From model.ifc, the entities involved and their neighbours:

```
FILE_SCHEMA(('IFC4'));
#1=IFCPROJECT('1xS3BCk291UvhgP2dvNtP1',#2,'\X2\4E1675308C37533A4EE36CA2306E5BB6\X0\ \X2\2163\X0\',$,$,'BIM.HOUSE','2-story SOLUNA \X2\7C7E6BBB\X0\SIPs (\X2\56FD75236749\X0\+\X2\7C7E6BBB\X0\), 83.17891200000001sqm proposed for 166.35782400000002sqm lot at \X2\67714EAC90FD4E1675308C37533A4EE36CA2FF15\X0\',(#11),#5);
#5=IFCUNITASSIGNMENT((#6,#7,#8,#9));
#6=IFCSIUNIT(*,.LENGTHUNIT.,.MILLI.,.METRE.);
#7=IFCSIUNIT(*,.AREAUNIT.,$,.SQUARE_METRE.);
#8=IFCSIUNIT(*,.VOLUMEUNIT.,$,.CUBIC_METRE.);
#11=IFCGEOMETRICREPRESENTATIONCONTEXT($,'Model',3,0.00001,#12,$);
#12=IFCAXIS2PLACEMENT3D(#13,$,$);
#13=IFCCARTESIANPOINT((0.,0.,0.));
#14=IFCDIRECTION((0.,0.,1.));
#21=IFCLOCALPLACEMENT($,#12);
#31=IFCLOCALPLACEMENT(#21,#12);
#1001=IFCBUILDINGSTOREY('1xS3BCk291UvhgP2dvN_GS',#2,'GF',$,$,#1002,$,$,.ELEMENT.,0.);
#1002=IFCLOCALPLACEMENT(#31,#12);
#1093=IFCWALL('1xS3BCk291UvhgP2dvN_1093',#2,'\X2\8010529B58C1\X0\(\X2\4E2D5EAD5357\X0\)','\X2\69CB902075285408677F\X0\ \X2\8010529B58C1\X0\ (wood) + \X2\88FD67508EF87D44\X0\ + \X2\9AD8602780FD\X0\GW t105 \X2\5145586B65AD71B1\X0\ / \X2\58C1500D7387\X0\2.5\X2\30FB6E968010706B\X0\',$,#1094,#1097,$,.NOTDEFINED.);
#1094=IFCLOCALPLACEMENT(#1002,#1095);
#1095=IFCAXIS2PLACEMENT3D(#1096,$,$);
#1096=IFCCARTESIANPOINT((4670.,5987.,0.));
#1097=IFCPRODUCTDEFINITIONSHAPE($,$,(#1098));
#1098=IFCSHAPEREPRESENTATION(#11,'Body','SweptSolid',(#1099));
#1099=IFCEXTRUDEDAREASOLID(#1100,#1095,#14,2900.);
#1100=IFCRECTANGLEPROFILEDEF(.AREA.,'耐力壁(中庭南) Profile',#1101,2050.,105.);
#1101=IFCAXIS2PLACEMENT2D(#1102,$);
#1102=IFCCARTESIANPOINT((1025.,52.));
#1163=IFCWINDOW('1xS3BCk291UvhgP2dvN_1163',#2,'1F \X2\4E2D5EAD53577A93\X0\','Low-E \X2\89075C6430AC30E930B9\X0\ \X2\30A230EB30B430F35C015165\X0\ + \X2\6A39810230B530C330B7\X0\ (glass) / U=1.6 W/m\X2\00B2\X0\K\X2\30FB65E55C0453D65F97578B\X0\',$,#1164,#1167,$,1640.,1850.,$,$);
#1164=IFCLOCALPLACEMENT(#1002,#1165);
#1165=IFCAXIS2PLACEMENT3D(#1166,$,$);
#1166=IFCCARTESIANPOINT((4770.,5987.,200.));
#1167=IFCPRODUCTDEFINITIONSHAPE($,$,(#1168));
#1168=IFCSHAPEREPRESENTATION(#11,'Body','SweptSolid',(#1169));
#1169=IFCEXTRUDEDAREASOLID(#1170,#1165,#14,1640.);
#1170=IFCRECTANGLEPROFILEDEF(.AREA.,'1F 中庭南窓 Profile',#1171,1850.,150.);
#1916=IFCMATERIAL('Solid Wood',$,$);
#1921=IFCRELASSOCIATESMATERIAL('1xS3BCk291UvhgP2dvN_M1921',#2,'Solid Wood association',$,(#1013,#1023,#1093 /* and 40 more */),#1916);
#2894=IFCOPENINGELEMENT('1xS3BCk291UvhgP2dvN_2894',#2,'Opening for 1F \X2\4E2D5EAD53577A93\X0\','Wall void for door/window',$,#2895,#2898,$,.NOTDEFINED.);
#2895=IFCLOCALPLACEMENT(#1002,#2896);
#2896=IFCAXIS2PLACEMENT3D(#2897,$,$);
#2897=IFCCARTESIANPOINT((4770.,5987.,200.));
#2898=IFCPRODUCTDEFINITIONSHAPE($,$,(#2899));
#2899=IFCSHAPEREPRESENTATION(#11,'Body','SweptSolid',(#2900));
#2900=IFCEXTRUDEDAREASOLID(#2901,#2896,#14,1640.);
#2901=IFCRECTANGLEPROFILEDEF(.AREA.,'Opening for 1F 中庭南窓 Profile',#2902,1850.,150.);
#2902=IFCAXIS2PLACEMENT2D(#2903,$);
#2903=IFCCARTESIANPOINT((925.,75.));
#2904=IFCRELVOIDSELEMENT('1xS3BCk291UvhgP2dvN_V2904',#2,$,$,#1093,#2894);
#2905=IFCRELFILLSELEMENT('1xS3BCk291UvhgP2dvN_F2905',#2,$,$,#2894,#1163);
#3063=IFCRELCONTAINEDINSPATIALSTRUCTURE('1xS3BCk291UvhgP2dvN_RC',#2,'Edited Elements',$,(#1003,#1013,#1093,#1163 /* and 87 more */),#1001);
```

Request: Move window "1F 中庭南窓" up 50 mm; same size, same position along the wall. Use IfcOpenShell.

```python
import numpy as np
import ifcopenshell
import ifcopenshell.api.geometry
import ifcopenshell.util.placement
import ifcopenshell.util.unit

model = ifcopenshell.open("model.ifc")
unit_scale = ifcopenshell.util.unit.calculate_unit_scale(model)

window = model.by_id(1163)
opening = window.FillsVoids[0].RelatingOpeningElement
dz = 0.05 / unit_scale

shift = np.array([0.0, 0.0, dz])
# The window is not placed relative to its opening, so move both.
for product in (opening, window):
    matrix = ifcopenshell.util.placement.get_local_placement(product.ObjectPlacement)
    matrix[:3, 3] += shift
    ifcopenshell.api.geometry.edit_object_placement(model, product=product, matrix=matrix, is_si=False)

print(f"moved by {dz * unit_scale:+.3f} m")

model.write("model_updated.ifc")
```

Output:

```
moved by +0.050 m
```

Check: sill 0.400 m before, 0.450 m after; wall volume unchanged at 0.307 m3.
